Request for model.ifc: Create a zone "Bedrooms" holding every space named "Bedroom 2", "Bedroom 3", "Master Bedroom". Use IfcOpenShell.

First a look at what the model holds.

```python
import ifcopenshell

model = ifcopenshell.open("model.ifc")
print(model.schema)
seen = {}
for space in model.by_type("IfcSpace"):
    seen[space.LongName] = seen.get(space.LongName, 0) + 1
for name, count in sorted(seen.items(), key=str):
    print(count, "x", name)
print("zones:", [z.Name for z in model.by_type("IfcZone")][:20])
```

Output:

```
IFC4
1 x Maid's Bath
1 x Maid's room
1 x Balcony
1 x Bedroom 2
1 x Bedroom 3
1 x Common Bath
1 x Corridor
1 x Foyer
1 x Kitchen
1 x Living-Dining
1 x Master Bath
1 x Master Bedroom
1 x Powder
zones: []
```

```python
import ifcopenshell
import ifcopenshell.api.group
import ifcopenshell.api.root

model = ifcopenshell.open("model.ifc")

names = {"Bedroom 2", "Bedroom 3", "Master Bedroom"}
spaces = [s for s in model.by_type("IfcSpace") if s.LongName in names]

zone = ifcopenshell.api.root.create_entity(model, ifc_class="IfcZone", name="Bedrooms")
ifcopenshell.api.group.assign_group(model, products=spaces, group=zone)
print(len(spaces), "spaces in", zone.Name)

model.write("model_updated.ifc")
```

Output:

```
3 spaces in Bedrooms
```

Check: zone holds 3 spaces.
